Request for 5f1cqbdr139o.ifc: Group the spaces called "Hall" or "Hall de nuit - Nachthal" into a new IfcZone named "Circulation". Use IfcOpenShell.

First a look at what the model holds.

```python
import ifcopenshell

model = ifcopenshell.open("5f1cqbdr139o.ifc")
print(model.schema)
seen = {}
for space in model.by_type("IfcSpace"):
    seen[space.LongName] = seen.get(space.LongName, 0) + 1
for name, count in sorted(seen.items(), key=str):
    print(count, "x", name)
print("zones:", [z.Name for z in model.by_type("IfcZone")][:20])
```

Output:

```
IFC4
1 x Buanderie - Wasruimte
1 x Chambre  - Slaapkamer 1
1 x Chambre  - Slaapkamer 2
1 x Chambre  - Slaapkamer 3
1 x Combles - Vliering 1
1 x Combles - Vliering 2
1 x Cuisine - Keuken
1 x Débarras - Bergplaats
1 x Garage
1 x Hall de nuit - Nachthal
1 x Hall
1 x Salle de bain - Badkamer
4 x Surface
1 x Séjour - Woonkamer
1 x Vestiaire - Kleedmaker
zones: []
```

```python
import ifcopenshell
import ifcopenshell.api.group
import ifcopenshell.api.root

model = ifcopenshell.open("5f1cqbdr139o.ifc")

names = {"Hall", "Hall de nuit - Nachthal"}
spaces = [s for s in model.by_type("IfcSpace") if s.LongName in names]

zone = ifcopenshell.api.root.create_entity(model, ifc_class="IfcZone", name="Circulation")
ifcopenshell.api.group.assign_group(model, products=spaces, group=zone)
print(len(spaces), "spaces in", zone.Name)

model.write("5f1cqbdr139o-out.ifc")
```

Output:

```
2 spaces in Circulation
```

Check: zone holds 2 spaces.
